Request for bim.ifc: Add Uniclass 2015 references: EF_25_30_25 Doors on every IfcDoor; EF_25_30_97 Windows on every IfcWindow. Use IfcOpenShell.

First a look at what the model holds.

```python
import ifcopenshell

model = ifcopenshell.open("bim.ifc")
print(model.schema)
print("classifications:", [c.Name for c in model.by_type("IfcClassification")])
for ifc_class in ("IfcDoor", "IfcRoof", "IfcStair", "IfcWall", "IfcWindow"):
    print(ifc_class, len(model.by_type(ifc_class)))
```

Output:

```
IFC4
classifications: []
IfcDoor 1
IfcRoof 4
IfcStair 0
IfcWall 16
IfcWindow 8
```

```python
import ifcopenshell
import ifcopenshell.api.classification

model = ifcopenshell.open("bim.ifc")

system = ifcopenshell.api.classification.add_classification(model, classification="Uniclass 2015")

codes = {
    "IfcDoor": ("EF_25_30_25", "Doors"),
    "IfcWindow": ("EF_25_30_97", "Windows"),
}
for ifc_class, (code, name) in codes.items():
    products = model.by_type(ifc_class)
    ifcopenshell.api.classification.add_reference(
        model, products=products, classification=system, identification=code, name=name
    )
    print(code, len(products))

model.write("bim_v2.ifc")
```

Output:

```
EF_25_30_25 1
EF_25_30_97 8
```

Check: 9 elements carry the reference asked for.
